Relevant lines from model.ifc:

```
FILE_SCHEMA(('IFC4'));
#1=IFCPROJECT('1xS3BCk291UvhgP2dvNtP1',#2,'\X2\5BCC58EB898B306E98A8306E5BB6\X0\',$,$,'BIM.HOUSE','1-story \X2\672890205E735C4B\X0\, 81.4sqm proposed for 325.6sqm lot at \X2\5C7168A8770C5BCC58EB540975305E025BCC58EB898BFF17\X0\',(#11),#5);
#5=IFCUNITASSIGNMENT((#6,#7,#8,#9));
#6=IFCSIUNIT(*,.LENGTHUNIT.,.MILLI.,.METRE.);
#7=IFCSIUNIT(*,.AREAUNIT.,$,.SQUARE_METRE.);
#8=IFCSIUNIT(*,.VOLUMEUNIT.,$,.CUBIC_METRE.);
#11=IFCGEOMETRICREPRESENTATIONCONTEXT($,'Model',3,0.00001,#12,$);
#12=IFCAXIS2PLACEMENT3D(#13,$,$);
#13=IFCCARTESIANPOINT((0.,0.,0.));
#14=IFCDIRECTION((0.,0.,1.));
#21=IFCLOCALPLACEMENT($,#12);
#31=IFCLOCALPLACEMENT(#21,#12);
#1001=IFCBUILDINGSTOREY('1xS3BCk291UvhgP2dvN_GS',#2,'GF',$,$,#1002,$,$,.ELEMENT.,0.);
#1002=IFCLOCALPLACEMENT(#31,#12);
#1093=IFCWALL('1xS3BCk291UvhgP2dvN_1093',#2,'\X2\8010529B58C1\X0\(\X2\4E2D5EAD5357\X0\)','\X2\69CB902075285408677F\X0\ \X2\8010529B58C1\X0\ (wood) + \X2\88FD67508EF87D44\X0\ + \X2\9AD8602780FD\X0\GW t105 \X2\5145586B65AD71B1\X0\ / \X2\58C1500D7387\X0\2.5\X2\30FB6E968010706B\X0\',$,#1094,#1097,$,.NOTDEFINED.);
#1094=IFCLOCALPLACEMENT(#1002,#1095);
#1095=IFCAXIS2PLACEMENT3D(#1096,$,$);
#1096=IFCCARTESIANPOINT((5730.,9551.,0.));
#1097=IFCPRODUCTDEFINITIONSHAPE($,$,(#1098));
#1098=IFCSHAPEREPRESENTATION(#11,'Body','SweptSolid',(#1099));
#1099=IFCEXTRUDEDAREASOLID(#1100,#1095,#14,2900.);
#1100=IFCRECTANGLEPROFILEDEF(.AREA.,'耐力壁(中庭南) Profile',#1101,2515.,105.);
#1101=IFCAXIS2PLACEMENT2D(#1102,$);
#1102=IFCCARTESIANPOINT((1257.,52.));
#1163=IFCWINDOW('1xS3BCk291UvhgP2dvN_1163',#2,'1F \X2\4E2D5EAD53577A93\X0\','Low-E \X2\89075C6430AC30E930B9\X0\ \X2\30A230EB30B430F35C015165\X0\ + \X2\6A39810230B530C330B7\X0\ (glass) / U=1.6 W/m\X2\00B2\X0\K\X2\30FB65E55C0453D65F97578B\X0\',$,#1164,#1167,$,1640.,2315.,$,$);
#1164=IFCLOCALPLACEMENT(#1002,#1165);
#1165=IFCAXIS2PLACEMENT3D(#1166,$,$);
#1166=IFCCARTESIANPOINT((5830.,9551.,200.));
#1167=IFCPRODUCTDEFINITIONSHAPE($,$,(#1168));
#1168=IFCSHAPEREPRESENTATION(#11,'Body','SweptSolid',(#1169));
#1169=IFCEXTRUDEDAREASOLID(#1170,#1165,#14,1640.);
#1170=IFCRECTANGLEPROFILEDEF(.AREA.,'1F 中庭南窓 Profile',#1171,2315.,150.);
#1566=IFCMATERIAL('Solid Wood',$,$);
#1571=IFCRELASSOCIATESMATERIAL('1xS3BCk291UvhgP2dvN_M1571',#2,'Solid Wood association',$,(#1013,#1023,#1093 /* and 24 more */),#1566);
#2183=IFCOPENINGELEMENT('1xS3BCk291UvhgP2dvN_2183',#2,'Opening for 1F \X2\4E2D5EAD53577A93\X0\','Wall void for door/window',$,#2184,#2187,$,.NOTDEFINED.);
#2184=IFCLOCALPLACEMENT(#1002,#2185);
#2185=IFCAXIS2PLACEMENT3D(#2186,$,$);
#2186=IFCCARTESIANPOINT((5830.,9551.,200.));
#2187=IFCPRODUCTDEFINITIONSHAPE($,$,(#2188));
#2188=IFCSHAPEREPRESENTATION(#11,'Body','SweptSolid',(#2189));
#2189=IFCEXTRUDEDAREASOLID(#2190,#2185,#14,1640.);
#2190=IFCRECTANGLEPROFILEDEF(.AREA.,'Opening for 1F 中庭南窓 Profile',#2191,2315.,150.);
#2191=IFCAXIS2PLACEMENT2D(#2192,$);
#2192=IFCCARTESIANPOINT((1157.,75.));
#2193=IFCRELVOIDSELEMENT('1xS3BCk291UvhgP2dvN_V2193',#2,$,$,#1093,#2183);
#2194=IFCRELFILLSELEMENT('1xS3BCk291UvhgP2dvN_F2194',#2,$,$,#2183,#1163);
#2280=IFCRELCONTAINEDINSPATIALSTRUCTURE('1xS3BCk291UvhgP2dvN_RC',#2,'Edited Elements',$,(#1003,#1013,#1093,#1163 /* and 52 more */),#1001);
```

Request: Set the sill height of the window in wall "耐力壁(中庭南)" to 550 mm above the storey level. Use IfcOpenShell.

```python
import numpy as np
import ifcopenshell
import ifcopenshell.api.geometry
import ifcopenshell.geom
import ifcopenshell.util.element
import ifcopenshell.util.placement
import ifcopenshell.util.shape
import ifcopenshell.util.unit

model = ifcopenshell.open("model.ifc")
unit_scale = ifcopenshell.util.unit.calculate_unit_scale(model)

window = model.by_guid("1xS3BCk291UvhgP2dvN_1163")
opening = window.FillsVoids[0].RelatingOpeningElement
storey = ifcopenshell.util.element.get_container(window, ifc_class="IfcBuildingStorey")
level = ifcopenshell.util.placement.get_local_placement(storey.ObjectPlacement)[2, 3]

# The opening's origin need not be at the sill, so measure its lowest point.
shape = ifcopenshell.geom.create_shape(ifcopenshell.geom.settings(), opening)
bottom = ifcopenshell.util.shape.get_shape_bottom_elevation(shape, shape.geometry) / unit_scale
dz = level + 0.55 / unit_scale - bottom

shift = np.array([0.0, 0.0, dz])
# The window is not placed relative to its opening, so move both.
for product in (opening, window):
    matrix = ifcopenshell.util.placement.get_local_placement(product.ObjectPlacement)
    matrix[:3, 3] += shift
    ifcopenshell.api.geometry.edit_object_placement(model, product=product, matrix=matrix, is_si=False)

print(f"moved by {dz * unit_scale:+.3f} m")

model.write("model-out.ifc")
```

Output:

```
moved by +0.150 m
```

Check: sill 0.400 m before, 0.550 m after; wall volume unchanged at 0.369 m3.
